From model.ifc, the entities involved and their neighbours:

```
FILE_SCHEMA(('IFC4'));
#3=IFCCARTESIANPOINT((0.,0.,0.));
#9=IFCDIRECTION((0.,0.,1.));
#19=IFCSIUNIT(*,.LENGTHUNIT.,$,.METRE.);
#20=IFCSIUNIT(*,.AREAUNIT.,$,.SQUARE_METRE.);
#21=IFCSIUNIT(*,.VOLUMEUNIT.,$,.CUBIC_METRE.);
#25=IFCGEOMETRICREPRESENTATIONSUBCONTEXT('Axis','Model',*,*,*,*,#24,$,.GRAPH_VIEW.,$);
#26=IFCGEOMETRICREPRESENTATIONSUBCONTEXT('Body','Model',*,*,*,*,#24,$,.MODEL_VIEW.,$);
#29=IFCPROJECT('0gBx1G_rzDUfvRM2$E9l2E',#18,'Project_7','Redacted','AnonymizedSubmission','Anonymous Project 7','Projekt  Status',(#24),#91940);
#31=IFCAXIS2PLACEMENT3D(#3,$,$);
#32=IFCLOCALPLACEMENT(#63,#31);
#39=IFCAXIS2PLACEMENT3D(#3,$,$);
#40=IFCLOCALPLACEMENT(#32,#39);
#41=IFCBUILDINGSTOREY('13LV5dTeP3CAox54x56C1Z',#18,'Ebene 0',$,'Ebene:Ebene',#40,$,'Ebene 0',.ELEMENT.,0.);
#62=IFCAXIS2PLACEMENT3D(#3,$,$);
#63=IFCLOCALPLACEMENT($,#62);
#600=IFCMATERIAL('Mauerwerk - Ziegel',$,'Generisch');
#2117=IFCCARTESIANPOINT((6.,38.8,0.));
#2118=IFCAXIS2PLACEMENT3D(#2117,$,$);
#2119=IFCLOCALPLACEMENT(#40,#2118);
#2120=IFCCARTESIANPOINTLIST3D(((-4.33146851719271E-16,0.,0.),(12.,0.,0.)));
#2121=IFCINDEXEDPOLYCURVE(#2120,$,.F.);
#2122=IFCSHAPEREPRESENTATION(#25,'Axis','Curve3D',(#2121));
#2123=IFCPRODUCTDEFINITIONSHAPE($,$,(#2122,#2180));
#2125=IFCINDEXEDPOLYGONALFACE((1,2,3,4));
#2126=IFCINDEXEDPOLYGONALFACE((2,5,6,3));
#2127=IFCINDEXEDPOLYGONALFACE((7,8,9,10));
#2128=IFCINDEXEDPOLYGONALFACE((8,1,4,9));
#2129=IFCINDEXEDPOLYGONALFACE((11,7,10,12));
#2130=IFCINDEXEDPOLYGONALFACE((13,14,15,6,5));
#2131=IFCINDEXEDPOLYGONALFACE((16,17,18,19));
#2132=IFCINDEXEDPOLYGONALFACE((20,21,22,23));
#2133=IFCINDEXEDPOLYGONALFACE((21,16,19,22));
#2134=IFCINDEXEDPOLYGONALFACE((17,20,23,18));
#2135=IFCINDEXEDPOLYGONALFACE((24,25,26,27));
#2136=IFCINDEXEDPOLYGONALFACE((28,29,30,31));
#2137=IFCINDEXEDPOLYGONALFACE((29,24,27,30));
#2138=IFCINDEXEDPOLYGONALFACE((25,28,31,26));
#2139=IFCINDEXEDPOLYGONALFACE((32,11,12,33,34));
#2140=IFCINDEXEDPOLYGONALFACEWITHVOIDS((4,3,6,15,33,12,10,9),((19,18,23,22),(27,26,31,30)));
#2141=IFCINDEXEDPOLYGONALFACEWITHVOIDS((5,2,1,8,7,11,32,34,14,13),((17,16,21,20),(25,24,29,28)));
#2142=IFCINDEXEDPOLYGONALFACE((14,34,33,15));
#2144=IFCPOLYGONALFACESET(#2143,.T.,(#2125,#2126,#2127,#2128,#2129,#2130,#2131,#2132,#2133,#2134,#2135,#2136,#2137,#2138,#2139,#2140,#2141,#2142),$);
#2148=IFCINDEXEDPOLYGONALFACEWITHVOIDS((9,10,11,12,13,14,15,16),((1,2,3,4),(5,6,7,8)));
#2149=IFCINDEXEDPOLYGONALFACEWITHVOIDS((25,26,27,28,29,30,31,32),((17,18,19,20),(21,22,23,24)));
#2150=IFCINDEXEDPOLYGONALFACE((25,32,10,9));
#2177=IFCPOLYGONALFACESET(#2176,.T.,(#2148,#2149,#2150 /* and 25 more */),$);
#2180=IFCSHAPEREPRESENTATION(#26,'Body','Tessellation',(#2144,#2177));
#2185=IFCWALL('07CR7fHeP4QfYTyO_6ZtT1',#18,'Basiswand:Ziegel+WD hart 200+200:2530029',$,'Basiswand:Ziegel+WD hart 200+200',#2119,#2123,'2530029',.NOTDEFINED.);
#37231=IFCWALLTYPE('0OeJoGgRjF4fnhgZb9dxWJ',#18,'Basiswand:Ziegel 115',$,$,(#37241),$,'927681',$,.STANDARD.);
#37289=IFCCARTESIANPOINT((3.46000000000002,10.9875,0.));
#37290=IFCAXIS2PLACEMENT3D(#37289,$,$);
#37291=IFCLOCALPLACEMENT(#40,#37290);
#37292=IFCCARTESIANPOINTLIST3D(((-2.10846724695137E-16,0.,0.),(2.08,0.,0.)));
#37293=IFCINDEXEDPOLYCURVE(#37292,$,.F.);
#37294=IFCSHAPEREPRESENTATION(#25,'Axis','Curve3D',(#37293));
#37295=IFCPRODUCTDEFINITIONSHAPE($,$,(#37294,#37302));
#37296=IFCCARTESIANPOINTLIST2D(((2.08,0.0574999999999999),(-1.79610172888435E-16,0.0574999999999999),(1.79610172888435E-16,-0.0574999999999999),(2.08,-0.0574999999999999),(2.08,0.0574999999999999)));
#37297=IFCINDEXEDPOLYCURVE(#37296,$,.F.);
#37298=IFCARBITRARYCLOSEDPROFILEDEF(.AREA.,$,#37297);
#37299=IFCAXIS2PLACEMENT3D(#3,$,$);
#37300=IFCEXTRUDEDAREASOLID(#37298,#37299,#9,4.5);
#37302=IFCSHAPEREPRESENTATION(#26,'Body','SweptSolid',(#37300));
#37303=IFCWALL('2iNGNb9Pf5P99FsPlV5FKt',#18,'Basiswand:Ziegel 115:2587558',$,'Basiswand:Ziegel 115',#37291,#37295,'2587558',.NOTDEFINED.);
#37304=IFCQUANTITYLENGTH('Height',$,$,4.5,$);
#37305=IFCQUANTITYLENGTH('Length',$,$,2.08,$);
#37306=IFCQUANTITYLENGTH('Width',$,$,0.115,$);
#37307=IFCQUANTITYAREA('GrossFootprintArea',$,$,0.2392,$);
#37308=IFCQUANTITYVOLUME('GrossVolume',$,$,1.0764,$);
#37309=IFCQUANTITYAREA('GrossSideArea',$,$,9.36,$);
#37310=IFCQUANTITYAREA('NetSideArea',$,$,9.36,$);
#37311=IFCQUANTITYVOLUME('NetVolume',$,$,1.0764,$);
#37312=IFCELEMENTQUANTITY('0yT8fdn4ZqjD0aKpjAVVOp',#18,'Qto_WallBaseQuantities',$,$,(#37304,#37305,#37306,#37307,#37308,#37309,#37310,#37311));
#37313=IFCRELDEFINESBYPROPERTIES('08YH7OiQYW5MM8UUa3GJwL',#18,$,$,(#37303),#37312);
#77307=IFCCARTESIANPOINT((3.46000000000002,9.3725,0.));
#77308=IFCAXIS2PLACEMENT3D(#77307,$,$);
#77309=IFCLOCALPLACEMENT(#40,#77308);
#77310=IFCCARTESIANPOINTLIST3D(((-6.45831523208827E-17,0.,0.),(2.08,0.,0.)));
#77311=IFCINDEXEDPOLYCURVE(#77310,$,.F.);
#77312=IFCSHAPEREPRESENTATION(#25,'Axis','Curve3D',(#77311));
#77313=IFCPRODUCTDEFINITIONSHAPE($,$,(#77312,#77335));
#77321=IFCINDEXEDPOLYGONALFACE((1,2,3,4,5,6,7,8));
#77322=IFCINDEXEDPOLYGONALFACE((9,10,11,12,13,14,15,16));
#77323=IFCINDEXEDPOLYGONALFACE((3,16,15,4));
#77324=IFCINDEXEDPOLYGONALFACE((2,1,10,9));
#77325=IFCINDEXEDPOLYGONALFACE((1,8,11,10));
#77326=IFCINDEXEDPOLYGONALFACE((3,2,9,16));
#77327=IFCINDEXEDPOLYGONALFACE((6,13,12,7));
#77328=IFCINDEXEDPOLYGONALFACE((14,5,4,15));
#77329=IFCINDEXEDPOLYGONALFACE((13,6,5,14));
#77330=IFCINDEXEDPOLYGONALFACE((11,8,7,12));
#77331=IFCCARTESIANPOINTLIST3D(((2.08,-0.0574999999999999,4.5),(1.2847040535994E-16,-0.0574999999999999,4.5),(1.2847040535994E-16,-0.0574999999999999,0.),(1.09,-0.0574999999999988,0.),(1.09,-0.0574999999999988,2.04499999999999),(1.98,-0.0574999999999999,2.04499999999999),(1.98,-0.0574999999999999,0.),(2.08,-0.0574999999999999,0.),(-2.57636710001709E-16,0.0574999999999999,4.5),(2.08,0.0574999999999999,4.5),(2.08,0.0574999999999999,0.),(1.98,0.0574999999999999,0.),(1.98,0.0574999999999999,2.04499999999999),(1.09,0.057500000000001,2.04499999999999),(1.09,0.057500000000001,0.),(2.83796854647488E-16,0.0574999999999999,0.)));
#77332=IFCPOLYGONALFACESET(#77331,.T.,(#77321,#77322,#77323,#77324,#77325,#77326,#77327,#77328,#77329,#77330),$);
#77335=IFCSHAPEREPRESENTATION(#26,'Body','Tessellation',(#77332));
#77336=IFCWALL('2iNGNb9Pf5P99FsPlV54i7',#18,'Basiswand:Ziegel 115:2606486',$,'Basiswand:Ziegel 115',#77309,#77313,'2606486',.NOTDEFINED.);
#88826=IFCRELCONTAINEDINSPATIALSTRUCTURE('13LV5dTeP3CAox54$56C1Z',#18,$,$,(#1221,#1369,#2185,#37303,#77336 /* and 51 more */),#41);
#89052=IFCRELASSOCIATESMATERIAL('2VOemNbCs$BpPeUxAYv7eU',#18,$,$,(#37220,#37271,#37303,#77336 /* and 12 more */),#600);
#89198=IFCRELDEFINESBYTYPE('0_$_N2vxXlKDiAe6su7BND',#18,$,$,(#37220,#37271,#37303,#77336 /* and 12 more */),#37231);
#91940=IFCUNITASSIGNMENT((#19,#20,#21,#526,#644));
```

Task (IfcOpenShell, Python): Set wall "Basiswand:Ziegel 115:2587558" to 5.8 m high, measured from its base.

```python
import ifcopenshell
import ifcopenshell.api.pset
import ifcopenshell.geom
import ifcopenshell.util.element
import ifcopenshell.util.representation
import ifcopenshell.util.shape
import ifcopenshell.util.unit

model = ifcopenshell.open("model.ifc")
unit_scale = ifcopenshell.util.unit.calculate_unit_scale(model)
area_scale = ifcopenshell.util.unit.calculate_unit_scale(model, "AREAUNIT")
volume_scale = ifcopenshell.util.unit.calculate_unit_scale(model, "VOLUMEUNIT")
settings = ifcopenshell.geom.settings()


def volume(element):
    """Net volume in cubic metres, openings subtracted."""
    shape = ifcopenshell.geom.create_shape(settings, element)
    return ifcopenshell.util.shape.get_volume(shape.geometry)


wall = model.by_guid("2iNGNb9Pf5P99FsPlV5FKt")
before = volume(wall)

body = ifcopenshell.util.representation.get_representation(wall, "Model", "Body")
solid = body.Items[0]
old_height = solid.Depth
solid.Depth = 5.8 / unit_scale
after = volume(wall)
thickness = 0.115  # wall thickness in metres

# Update the stored height, areas and volumes.
qto = model.by_id(ifcopenshell.util.element.get_pset(wall, "Qto_WallBaseQuantities", should_inherit=False)["id"])
ifcopenshell.api.pset.edit_qto(model, qto=qto, properties={
    "Height": solid.Depth,
    "GrossVolume": ifcopenshell.util.element.get_pset(wall, "Qto_WallBaseQuantities", "GrossVolume") * solid.Depth / old_height,
    "GrossSideArea": ifcopenshell.util.element.get_pset(wall, "Qto_WallBaseQuantities", "GrossSideArea") * solid.Depth / old_height,
    "NetSideArea": after / thickness / area_scale,
    "NetVolume": after / volume_scale,
})

print(f"height {old_height:g} -> {solid.Depth:g}, volume {before:.3f} -> {after:.3f} m3")

model.write("model_edited.ifc")
```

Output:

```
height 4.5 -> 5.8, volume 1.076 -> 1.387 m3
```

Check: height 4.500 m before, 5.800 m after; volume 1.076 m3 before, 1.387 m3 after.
